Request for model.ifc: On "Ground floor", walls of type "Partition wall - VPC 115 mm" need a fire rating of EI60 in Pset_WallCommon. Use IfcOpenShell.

First a look at what the model holds.

```python
import ifcopenshell
import ifcopenshell.util.element

model = ifcopenshell.open("model.ifc")
print(model.schema)
storey = next(s for s in model.by_type("IfcBuildingStorey") if s.Name == "Ground floor")
walls = [e for e in ifcopenshell.util.element.get_decomposition(storey) if e.is_a("IfcWall")]
seen = {}
for e in walls:
    element_type = ifcopenshell.util.element.get_type(e)
    key = (element_type.Name if element_type != e and element_type else None, ifcopenshell.util.element.get_pset(e, "Pset_WallCommon", "FireRating"))
    seen[key] = seen.get(key, 0) + 1
for (name, value), count in sorted(seen.items(), key=str):
    print(count, "x", name, "|", value)
```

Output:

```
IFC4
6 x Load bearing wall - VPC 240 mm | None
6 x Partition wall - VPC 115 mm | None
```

```python
import ifcopenshell
import ifcopenshell.api.pset
import ifcopenshell.util.element

model = ifcopenshell.open("model.ifc")

storey = next(s for s in model.by_type("IfcBuildingStorey") if s.Name == "Ground floor")
walls = [e for e in ifcopenshell.util.element.get_decomposition(storey) if e.is_a("IfcWall")]

count = 0
for e in walls:
    element_type = ifcopenshell.util.element.get_type(e)
    if element_type in (None, e) or element_type.Name != "Partition wall - VPC 115 mm":
        continue
    # add_pset returns the element's existing set when there is one.
    pset = ifcopenshell.api.pset.add_pset(model, product=e, name="Pset_WallCommon")
    ifcopenshell.api.pset.edit_pset(model, pset=pset, properties={"FireRating": "EI60"})
    count += 1

print(count, "walls updated")

model.write("model_updated.ifc")
```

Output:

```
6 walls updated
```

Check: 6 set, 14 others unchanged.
